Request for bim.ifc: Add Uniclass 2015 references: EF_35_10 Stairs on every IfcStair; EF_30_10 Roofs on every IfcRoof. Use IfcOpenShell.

First a look at what the model holds.

```python
import ifcopenshell

model = ifcopenshell.open("bim.ifc")
print(model.schema)
print("classifications:", [c.Name for c in model.by_type("IfcClassification")])
for ifc_class in ("IfcDoor", "IfcRoof", "IfcStair", "IfcWall", "IfcWindow"):
    print(ifc_class, len(model.by_type(ifc_class)))
```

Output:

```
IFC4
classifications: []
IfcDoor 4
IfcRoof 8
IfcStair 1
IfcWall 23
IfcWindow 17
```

```python
import ifcopenshell
import ifcopenshell.api.classification

model = ifcopenshell.open("bim.ifc")

system = ifcopenshell.api.classification.add_classification(model, classification="Uniclass 2015")

codes = {
    "IfcStair": ("EF_35_10", "Stairs"),
    "IfcRoof": ("EF_30_10", "Roofs"),
}
for ifc_class, (code, name) in codes.items():
    products = model.by_type(ifc_class)
    ifcopenshell.api.classification.add_reference(
        model, products=products, classification=system, identification=code, name=name
    )
    print(code, len(products))

model.write("bim_edited.ifc")
```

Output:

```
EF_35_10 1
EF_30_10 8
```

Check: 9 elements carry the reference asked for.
